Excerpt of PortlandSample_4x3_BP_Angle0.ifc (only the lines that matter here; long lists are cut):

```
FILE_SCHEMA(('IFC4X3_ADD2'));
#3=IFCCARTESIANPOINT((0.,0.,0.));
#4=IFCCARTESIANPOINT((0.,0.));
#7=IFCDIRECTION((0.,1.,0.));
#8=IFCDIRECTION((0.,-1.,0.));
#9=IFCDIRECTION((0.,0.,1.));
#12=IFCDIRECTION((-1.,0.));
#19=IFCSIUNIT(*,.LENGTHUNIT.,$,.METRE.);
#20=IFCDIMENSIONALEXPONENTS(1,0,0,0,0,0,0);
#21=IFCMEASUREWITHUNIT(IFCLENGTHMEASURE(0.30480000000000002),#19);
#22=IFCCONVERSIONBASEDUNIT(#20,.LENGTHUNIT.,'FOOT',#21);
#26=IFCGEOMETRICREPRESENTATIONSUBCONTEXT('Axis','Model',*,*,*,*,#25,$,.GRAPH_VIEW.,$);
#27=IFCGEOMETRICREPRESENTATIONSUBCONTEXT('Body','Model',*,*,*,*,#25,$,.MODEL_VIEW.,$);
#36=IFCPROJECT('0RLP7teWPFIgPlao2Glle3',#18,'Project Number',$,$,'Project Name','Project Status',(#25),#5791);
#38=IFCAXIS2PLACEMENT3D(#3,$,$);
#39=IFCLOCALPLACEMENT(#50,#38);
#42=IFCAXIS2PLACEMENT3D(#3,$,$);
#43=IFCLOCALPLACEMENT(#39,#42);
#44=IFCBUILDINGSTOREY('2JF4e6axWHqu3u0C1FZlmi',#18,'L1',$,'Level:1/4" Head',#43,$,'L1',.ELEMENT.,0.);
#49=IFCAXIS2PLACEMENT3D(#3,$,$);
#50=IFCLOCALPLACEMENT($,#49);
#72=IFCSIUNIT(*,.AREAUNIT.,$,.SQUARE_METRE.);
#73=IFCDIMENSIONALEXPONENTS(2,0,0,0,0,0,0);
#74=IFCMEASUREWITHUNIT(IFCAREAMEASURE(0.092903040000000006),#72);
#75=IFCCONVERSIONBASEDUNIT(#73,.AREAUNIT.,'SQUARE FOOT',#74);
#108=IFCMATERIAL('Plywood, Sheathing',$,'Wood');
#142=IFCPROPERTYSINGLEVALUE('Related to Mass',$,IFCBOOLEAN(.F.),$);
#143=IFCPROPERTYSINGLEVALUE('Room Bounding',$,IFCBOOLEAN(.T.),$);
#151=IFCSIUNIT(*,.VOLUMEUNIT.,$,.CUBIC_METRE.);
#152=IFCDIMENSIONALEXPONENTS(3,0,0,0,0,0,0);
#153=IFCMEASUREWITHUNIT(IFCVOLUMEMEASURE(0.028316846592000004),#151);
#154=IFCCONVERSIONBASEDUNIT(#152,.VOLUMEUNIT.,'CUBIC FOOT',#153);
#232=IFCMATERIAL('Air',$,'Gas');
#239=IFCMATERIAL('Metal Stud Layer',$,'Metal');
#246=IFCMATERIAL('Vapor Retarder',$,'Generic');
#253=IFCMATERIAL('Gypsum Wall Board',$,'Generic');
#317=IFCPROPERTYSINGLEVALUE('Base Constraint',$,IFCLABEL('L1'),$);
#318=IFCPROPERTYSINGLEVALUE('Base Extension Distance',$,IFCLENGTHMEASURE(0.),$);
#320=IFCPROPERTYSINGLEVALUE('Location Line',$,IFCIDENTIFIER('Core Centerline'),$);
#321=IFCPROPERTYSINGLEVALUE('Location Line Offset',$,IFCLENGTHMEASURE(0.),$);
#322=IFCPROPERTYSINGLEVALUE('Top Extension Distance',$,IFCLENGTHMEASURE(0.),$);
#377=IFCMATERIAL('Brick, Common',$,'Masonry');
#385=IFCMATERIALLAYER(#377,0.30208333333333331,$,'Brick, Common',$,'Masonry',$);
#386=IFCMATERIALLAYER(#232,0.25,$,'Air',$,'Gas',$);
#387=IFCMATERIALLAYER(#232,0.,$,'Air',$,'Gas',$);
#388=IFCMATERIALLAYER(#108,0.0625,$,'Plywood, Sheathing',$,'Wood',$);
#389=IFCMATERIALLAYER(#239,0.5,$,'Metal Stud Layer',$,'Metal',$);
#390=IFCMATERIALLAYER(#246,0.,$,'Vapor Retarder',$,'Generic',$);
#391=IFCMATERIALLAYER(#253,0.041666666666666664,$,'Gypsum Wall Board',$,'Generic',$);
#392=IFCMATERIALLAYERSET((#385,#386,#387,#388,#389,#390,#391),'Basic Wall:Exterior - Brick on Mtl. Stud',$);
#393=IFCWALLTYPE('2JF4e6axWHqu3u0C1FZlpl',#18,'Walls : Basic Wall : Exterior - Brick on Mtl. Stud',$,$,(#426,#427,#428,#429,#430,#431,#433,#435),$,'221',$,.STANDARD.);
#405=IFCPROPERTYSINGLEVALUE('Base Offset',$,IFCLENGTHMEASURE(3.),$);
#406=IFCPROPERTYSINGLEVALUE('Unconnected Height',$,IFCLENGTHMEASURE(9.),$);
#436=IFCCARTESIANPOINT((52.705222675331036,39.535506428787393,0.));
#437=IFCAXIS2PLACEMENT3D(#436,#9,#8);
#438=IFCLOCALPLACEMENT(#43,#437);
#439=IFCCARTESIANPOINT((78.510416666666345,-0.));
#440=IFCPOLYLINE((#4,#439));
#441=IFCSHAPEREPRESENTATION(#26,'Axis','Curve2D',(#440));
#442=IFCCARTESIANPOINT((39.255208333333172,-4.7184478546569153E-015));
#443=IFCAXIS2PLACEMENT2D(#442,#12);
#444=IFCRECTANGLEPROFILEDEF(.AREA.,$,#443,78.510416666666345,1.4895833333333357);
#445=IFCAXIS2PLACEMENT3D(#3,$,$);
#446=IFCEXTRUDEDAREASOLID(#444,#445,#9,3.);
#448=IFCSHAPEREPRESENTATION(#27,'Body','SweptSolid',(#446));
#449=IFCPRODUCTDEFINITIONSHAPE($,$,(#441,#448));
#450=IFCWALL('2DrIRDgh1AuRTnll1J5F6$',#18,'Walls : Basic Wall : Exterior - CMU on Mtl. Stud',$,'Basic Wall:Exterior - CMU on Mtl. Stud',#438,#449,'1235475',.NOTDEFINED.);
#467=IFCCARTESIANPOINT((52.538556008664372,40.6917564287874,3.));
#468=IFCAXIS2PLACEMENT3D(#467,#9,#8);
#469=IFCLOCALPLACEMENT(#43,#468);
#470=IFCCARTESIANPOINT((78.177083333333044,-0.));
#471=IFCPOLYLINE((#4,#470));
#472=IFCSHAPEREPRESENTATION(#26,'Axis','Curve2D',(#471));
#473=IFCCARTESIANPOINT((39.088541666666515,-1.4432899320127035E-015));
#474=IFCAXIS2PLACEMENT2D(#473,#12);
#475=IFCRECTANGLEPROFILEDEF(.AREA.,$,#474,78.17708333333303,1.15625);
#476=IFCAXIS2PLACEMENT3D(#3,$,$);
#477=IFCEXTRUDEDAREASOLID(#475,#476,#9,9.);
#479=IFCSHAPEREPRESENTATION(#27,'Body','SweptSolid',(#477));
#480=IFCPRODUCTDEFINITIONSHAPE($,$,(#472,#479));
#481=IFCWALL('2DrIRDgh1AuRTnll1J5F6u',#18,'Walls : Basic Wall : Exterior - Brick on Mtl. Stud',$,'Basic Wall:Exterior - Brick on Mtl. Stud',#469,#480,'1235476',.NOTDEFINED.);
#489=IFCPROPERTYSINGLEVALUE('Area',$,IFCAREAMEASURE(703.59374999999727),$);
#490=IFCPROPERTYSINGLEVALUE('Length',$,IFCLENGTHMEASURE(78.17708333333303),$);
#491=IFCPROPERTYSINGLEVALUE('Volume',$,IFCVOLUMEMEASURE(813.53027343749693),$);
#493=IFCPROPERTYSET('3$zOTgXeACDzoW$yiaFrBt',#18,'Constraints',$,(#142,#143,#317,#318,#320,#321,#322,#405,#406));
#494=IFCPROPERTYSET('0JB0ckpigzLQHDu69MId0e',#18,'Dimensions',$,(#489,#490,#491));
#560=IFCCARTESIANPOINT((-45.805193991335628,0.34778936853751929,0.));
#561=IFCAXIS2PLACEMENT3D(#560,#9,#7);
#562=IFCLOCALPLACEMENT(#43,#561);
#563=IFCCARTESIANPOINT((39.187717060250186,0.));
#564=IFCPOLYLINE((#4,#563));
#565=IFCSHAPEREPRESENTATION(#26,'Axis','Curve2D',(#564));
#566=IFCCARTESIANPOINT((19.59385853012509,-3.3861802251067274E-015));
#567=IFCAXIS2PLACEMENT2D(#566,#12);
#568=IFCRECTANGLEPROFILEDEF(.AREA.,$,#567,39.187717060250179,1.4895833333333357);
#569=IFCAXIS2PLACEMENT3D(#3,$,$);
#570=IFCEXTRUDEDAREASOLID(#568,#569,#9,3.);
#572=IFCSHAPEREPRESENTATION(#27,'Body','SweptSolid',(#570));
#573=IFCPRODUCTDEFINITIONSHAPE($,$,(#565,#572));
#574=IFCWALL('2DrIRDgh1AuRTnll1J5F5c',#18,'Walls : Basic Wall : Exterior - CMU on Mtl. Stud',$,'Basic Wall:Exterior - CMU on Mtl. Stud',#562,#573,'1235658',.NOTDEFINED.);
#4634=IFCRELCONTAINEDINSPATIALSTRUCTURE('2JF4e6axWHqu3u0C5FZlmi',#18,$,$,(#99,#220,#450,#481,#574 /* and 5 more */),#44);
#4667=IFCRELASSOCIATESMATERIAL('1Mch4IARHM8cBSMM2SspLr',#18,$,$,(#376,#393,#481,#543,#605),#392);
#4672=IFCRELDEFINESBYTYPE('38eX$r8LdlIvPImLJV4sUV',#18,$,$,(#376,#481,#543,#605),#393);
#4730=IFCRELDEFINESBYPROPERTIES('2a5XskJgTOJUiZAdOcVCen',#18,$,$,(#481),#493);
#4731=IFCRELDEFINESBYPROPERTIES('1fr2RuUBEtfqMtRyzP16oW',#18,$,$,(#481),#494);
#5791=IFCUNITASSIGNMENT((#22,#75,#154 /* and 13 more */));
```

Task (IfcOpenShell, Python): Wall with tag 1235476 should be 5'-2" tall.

```python
import ifcopenshell
import ifcopenshell.api.pset
import ifcopenshell.geom
import ifcopenshell.util.element
import ifcopenshell.util.representation
import ifcopenshell.util.shape
import ifcopenshell.util.unit

model = ifcopenshell.open("PortlandSample_4x3_BP_Angle0.ifc")
unit_scale = ifcopenshell.util.unit.calculate_unit_scale(model)
area_scale = ifcopenshell.util.unit.calculate_unit_scale(model, "AREAUNIT")
volume_scale = ifcopenshell.util.unit.calculate_unit_scale(model, "VOLUMEUNIT")
settings = ifcopenshell.geom.settings()


def volume(element):
    """Net volume in cubic metres, openings subtracted."""
    shape = ifcopenshell.geom.create_shape(settings, element)
    return ifcopenshell.util.shape.get_volume(shape.geometry)


wall = model.by_guid("2DrIRDgh1AuRTnll1J5F6u")
before = volume(wall)

body = ifcopenshell.util.representation.get_representation(wall, "Model", "Body")
solid = body.Items[0]
old_height = solid.Depth
solid.Depth = 62 * 0.0254 / unit_scale
after = volume(wall)
thickness = 0.3524  # wall thickness in metres

# Update the stored height, areas and volumes.
pset = model.by_id(ifcopenshell.util.element.get_pset(wall, "Constraints", should_inherit=False)["id"])
ifcopenshell.api.pset.edit_pset(model, pset=pset, properties={
    "Unconnected Height": model.create_entity("IfcLengthMeasure", solid.Depth),
})
pset = model.by_id(ifcopenshell.util.element.get_pset(wall, "Dimensions", should_inherit=False)["id"])
ifcopenshell.api.pset.edit_pset(model, pset=pset, properties={
    "Area": model.create_entity("IfcAreaMeasure", after / thickness / area_scale),
    "Volume": model.create_entity("IfcVolumeMeasure", after / volume_scale),
})

print(f"height {old_height:g} -> {solid.Depth:g}, volume {before:.3f} -> {after:.3f} m3")

model.write("PortlandSample_4x3_BP_Angle0_updated.ifc")
```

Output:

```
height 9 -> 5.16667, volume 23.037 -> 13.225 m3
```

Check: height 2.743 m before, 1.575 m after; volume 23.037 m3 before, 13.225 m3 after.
